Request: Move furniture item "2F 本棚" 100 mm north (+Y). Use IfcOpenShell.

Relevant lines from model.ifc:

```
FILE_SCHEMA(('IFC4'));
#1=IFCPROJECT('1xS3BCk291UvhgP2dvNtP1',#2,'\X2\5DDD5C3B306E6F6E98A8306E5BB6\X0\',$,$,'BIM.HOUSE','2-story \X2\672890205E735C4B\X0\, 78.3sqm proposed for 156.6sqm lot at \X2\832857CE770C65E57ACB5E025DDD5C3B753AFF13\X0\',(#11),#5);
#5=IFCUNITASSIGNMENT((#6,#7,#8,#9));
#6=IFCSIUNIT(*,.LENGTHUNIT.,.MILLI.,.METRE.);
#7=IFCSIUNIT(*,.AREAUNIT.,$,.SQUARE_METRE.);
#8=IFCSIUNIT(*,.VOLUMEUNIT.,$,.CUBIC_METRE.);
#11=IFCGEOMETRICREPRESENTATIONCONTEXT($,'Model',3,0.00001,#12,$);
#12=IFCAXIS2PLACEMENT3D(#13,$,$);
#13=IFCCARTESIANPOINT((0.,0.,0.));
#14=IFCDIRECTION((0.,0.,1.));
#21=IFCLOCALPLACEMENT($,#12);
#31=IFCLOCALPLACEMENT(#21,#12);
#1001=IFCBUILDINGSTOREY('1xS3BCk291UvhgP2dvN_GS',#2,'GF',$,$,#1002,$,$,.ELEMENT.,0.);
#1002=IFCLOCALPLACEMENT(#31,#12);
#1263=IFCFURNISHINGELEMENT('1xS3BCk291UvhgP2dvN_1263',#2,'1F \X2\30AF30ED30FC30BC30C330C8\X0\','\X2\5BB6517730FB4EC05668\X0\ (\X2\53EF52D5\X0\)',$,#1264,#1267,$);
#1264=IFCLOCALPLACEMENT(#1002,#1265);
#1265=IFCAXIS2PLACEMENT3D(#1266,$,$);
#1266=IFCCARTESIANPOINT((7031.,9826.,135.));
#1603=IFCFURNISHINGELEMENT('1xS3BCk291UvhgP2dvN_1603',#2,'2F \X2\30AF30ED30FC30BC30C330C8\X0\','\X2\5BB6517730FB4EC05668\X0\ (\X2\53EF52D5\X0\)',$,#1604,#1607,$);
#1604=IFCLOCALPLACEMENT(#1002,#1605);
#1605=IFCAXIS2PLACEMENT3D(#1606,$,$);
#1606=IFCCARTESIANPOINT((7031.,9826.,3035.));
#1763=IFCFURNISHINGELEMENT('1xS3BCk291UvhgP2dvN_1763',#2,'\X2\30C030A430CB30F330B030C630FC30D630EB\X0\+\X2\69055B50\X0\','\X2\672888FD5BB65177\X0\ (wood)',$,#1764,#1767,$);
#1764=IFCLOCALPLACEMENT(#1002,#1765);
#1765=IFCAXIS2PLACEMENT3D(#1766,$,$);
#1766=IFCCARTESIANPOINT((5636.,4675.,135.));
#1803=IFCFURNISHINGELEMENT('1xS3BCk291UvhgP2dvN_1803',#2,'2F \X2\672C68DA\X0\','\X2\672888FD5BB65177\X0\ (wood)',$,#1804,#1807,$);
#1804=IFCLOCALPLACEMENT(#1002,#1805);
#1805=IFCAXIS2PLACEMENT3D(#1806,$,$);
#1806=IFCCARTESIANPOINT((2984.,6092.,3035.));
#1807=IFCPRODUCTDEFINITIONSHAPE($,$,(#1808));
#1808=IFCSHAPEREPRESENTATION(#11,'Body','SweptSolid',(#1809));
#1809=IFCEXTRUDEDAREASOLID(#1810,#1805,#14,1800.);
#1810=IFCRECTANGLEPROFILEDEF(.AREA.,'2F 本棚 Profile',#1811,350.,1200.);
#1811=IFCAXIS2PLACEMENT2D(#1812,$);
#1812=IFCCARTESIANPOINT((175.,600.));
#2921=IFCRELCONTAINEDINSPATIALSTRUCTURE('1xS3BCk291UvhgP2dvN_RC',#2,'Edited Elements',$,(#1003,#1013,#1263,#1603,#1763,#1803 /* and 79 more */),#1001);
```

```python
import ifcopenshell
import ifcopenshell.api.geometry
import ifcopenshell.util.placement

model = ifcopenshell.open("model.ifc")

item = model.by_guid("1xS3BCk291UvhgP2dvN_1803")
matrix = ifcopenshell.util.placement.get_local_placement(item.ObjectPlacement)
matrix[1, 3] += 100.0
ifcopenshell.api.geometry.edit_object_placement(model, product=item, matrix=matrix, is_si=False)

print(ifcopenshell.util.placement.get_local_placement(item.ObjectPlacement).round(3) + 0.0)

model.write("model-out.ifc")
```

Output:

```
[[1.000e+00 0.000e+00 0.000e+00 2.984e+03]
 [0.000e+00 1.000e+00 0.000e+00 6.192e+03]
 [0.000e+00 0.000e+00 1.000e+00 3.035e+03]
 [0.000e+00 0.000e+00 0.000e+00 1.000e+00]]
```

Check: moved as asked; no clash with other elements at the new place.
